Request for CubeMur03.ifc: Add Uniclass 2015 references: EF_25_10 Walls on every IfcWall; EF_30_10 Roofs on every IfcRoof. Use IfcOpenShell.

First a look at what the model holds.

```python
import ifcopenshell

model = ifcopenshell.open("CubeMur03.ifc")
print(model.schema)
print("classifications:", [c.Name for c in model.by_type("IfcClassification")])
for ifc_class in ("IfcDoor", "IfcRoof", "IfcStair", "IfcWall", "IfcWindow"):
    print(ifc_class, len(model.by_type(ifc_class)))
```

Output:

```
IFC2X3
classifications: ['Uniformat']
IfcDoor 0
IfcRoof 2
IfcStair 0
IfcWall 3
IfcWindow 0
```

```python
import ifcopenshell
import ifcopenshell.api.classification

model = ifcopenshell.open("CubeMur03.ifc")

# IFC2X3 requires Source and Edition and has no link from the project to the system.
system = model.create_entity("IfcClassification", Source="NBS", Edition="2015", Name="Uniclass 2015")

codes = {
    "IfcWall": ("EF_25_10", "Walls"),
    "IfcRoof": ("EF_30_10", "Roofs"),
}
for ifc_class, (code, name) in codes.items():
    products = model.by_type(ifc_class)
    ifcopenshell.api.classification.add_reference(
        model, products=products, classification=system, identification=code, name=name
    )
    print(code, len(products))

model.write("CubeMur03_updated.ifc")
```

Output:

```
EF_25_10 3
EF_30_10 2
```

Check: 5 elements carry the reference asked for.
